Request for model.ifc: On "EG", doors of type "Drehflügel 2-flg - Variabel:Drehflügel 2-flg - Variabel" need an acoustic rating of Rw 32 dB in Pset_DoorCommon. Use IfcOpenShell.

First a look at what the model holds.

```python
import ifcopenshell
import ifcopenshell.util.element

model = ifcopenshell.open("model.ifc")
print(model.schema)
storey = next(s for s in model.by_type("IfcBuildingStorey") if s.Name == "EG")
doors = [e for e in ifcopenshell.util.element.get_decomposition(storey) if e.is_a("IfcDoor")]
seen = {}
for e in doors:
    element_type = ifcopenshell.util.element.get_type(e)
    key = (element_type.Name if element_type != e and element_type else None, ifcopenshell.util.element.get_pset(e, "Pset_DoorCommon", "AcousticRating"))
    seen[key] = seen.get(key, 0) + 1
for (name, value), count in sorted(seen.items(), key=str):
    print(count, "x", name, "|", value)
```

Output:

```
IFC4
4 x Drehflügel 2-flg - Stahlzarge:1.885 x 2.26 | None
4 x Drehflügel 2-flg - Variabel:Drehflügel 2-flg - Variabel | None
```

```python
import ifcopenshell
import ifcopenshell.api.pset
import ifcopenshell.util.element

model = ifcopenshell.open("model.ifc")

storey = next(s for s in model.by_type("IfcBuildingStorey") if s.Name == "EG")
doors = [e for e in ifcopenshell.util.element.get_decomposition(storey) if e.is_a("IfcDoor")]

count = 0
for e in doors:
    element_type = ifcopenshell.util.element.get_type(e)
    if element_type in (None, e) or element_type.Name != "Drehflügel 2-flg - Variabel:Drehflügel 2-flg - Variabel":
        continue
    # add_pset returns the element's existing set when there is one.
    pset = ifcopenshell.api.pset.add_pset(model, product=e, name="Pset_DoorCommon")
    ifcopenshell.api.pset.edit_pset(model, pset=pset, properties={"AcousticRating": "Rw 32 dB"})
    count += 1

print(count, "doors updated")

model.write("model_updated.ifc")
```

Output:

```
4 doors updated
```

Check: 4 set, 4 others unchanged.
